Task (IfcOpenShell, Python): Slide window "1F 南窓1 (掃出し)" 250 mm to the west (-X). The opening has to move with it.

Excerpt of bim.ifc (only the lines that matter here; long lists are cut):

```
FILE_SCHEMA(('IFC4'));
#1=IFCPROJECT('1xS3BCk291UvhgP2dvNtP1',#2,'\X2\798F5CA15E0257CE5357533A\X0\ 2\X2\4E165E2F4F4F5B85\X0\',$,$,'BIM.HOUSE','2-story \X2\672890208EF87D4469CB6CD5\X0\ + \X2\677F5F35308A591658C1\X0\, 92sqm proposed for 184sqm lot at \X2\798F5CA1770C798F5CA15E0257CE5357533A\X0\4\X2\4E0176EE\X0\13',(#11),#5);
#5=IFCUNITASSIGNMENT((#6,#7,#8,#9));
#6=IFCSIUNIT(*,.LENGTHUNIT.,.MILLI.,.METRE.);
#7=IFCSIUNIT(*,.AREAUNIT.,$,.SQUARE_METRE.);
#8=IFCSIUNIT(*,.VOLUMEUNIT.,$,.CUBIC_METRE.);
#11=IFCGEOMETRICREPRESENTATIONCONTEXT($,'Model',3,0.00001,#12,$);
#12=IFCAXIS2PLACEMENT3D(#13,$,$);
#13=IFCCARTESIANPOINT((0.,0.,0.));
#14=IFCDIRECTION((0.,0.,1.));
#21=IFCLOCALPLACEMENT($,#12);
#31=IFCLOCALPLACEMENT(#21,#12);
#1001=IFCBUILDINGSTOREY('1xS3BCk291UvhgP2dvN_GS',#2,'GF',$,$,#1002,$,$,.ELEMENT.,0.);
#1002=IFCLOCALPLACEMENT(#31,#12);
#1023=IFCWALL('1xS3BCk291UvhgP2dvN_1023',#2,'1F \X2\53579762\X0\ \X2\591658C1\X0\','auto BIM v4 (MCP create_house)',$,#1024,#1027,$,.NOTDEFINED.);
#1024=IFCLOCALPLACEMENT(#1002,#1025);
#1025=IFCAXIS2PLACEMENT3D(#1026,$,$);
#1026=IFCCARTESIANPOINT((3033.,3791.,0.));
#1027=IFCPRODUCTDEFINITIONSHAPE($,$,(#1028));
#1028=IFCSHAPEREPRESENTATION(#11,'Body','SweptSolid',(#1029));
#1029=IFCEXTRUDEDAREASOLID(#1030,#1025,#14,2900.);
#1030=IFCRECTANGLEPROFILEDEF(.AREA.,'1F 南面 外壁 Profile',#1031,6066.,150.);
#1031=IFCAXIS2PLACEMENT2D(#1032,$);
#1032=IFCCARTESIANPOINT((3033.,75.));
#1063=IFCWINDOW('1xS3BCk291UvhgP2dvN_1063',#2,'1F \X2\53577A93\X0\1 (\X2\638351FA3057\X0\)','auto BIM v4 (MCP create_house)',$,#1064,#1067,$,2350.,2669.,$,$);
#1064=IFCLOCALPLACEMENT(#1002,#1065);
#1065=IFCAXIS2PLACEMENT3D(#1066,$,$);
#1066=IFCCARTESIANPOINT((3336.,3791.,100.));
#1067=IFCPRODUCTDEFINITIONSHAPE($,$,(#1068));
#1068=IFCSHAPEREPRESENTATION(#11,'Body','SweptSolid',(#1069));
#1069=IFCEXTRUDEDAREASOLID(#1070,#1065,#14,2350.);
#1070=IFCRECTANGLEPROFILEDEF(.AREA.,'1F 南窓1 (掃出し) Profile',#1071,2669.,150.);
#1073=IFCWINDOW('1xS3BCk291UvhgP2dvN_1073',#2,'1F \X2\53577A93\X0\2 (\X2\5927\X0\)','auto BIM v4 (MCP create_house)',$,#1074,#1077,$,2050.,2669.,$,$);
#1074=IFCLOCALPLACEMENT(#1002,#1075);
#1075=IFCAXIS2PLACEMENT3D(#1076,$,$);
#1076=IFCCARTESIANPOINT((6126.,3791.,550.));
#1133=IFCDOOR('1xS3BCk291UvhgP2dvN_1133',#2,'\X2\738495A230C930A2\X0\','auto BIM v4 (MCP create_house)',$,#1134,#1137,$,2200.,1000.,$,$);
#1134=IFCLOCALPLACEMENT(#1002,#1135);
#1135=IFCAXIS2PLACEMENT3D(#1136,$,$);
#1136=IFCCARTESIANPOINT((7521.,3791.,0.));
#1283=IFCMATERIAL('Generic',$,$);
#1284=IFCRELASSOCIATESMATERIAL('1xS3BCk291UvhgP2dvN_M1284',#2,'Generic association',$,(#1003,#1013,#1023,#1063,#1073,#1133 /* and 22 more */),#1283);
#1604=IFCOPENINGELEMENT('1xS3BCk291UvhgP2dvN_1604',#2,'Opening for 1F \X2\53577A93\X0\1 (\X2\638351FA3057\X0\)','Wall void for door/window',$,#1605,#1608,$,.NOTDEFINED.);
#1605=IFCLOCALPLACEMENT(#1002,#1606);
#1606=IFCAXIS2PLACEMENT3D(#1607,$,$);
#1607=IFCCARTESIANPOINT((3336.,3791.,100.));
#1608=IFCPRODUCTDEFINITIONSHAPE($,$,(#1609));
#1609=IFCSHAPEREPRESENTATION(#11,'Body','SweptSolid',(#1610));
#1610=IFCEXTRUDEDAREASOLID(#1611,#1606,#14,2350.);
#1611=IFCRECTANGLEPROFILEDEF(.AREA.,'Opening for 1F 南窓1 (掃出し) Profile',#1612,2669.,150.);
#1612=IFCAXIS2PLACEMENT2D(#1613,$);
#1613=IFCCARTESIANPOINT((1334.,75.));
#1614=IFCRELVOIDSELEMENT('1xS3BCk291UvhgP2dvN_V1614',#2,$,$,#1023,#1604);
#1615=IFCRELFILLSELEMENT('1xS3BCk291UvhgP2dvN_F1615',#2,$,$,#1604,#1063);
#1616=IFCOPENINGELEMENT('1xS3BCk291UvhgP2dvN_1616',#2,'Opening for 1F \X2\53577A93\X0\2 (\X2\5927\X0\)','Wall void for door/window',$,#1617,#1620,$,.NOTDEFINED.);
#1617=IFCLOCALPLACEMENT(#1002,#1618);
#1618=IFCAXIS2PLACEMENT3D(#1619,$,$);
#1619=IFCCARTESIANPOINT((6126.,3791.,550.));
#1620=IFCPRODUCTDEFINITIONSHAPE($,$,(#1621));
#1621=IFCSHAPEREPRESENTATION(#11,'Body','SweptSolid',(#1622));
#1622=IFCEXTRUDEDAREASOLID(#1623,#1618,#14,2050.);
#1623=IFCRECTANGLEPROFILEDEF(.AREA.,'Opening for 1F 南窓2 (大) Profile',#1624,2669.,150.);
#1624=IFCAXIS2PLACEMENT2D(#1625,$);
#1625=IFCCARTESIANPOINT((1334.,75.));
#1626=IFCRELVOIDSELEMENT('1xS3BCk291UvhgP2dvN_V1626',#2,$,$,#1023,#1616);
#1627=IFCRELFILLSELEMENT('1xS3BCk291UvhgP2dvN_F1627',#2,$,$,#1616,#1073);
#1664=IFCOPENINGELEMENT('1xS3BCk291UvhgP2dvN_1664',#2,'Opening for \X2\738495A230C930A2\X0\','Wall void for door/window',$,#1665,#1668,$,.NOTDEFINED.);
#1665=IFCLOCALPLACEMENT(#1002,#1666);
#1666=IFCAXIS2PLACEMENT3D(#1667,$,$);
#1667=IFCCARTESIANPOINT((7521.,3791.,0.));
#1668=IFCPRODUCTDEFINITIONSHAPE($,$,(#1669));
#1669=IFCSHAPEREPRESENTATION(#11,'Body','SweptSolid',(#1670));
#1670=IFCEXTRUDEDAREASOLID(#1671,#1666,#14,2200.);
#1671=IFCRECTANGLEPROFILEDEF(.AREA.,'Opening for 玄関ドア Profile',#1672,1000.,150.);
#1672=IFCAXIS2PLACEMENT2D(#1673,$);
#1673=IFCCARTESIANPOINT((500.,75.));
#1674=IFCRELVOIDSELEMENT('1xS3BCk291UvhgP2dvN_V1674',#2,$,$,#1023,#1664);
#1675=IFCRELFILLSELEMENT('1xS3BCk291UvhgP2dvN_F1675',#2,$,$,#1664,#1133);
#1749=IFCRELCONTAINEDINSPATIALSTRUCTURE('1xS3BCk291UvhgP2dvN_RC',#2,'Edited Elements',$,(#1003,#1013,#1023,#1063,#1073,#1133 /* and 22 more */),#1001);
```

```python
import ifcopenshell
import ifcopenshell.api.geometry
import ifcopenshell.util.placement
import ifcopenshell.util.unit

model = ifcopenshell.open("bim.ifc")
unit_scale = ifcopenshell.util.unit.calculate_unit_scale(model)

window = model.by_id(1063)
opening = window.FillsVoids[0].RelatingOpeningElement
wall = opening.VoidsElements[0].RelatingBuildingElement

wall_matrix = ifcopenshell.util.placement.get_local_placement(wall.ObjectPlacement)
shift = wall_matrix[:3, 0] * -0.25 / unit_scale
before = ifcopenshell.util.placement.get_local_placement(window.ObjectPlacement)[:3, 3].copy()

# The window is not placed relative to its opening, so move both.
for product in (opening, window):
    matrix = ifcopenshell.util.placement.get_local_placement(product.ObjectPlacement)
    matrix[:3, 3] += shift
    ifcopenshell.api.geometry.edit_object_placement(model, product=product, matrix=matrix, is_si=False)

after = ifcopenshell.util.placement.get_local_placement(window.ObjectPlacement)[:3, 3]
print("window moved by", (after - before).round(3) + 0.0)

model.write("bim_edited.ifc")
```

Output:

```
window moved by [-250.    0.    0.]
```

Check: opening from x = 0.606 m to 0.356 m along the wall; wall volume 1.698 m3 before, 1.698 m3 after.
